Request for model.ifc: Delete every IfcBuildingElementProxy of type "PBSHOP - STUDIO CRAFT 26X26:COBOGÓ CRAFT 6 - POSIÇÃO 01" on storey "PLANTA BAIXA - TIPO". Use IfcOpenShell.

First a look at what the model holds.

```python
import ifcopenshell
import ifcopenshell.util.element

model = ifcopenshell.open("model.ifc")
print(model.schema)
storey = next(s for s in model.by_type("IfcBuildingStorey") if s.Name == "PLANTA BAIXA - TIPO")
proxies = [e for e in ifcopenshell.util.element.get_decomposition(storey) if e.is_a("IfcBuildingElementProxy")]
seen = {}
for e in proxies:
    element_type = ifcopenshell.util.element.get_type(e)
    name = element_type.Name if element_type not in (None, e) else None
    seen[name] = seen.get(name, 0) + 1
for name, count in sorted(seen.items(), key=str):
    print(count, "x", name)
```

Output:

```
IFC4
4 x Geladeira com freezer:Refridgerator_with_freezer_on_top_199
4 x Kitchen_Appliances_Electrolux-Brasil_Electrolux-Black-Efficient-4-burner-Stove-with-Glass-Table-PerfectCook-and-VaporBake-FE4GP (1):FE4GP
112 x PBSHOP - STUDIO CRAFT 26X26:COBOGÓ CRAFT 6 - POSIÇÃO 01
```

```python
import ifcopenshell
import ifcopenshell.api.root
import ifcopenshell.util.element

model = ifcopenshell.open("model.ifc")

storey = next(s for s in model.by_type("IfcBuildingStorey") if s.Name == "PLANTA BAIXA - TIPO")
proxies = [e for e in ifcopenshell.util.element.get_decomposition(storey) if e.is_a("IfcBuildingElementProxy")]
targets = [e for e in proxies if (t := ifcopenshell.util.element.get_type(e)) not in (None, e) and t.Name == "PBSHOP - STUDIO CRAFT 26X26:COBOGÓ CRAFT 6 - POSIÇÃO 01"]

for e in targets:
    ifcopenshell.api.root.remove_product(model, product=e)
print(len(targets), "removed")

model.write("model_updated.ifc")
```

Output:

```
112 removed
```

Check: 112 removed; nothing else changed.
